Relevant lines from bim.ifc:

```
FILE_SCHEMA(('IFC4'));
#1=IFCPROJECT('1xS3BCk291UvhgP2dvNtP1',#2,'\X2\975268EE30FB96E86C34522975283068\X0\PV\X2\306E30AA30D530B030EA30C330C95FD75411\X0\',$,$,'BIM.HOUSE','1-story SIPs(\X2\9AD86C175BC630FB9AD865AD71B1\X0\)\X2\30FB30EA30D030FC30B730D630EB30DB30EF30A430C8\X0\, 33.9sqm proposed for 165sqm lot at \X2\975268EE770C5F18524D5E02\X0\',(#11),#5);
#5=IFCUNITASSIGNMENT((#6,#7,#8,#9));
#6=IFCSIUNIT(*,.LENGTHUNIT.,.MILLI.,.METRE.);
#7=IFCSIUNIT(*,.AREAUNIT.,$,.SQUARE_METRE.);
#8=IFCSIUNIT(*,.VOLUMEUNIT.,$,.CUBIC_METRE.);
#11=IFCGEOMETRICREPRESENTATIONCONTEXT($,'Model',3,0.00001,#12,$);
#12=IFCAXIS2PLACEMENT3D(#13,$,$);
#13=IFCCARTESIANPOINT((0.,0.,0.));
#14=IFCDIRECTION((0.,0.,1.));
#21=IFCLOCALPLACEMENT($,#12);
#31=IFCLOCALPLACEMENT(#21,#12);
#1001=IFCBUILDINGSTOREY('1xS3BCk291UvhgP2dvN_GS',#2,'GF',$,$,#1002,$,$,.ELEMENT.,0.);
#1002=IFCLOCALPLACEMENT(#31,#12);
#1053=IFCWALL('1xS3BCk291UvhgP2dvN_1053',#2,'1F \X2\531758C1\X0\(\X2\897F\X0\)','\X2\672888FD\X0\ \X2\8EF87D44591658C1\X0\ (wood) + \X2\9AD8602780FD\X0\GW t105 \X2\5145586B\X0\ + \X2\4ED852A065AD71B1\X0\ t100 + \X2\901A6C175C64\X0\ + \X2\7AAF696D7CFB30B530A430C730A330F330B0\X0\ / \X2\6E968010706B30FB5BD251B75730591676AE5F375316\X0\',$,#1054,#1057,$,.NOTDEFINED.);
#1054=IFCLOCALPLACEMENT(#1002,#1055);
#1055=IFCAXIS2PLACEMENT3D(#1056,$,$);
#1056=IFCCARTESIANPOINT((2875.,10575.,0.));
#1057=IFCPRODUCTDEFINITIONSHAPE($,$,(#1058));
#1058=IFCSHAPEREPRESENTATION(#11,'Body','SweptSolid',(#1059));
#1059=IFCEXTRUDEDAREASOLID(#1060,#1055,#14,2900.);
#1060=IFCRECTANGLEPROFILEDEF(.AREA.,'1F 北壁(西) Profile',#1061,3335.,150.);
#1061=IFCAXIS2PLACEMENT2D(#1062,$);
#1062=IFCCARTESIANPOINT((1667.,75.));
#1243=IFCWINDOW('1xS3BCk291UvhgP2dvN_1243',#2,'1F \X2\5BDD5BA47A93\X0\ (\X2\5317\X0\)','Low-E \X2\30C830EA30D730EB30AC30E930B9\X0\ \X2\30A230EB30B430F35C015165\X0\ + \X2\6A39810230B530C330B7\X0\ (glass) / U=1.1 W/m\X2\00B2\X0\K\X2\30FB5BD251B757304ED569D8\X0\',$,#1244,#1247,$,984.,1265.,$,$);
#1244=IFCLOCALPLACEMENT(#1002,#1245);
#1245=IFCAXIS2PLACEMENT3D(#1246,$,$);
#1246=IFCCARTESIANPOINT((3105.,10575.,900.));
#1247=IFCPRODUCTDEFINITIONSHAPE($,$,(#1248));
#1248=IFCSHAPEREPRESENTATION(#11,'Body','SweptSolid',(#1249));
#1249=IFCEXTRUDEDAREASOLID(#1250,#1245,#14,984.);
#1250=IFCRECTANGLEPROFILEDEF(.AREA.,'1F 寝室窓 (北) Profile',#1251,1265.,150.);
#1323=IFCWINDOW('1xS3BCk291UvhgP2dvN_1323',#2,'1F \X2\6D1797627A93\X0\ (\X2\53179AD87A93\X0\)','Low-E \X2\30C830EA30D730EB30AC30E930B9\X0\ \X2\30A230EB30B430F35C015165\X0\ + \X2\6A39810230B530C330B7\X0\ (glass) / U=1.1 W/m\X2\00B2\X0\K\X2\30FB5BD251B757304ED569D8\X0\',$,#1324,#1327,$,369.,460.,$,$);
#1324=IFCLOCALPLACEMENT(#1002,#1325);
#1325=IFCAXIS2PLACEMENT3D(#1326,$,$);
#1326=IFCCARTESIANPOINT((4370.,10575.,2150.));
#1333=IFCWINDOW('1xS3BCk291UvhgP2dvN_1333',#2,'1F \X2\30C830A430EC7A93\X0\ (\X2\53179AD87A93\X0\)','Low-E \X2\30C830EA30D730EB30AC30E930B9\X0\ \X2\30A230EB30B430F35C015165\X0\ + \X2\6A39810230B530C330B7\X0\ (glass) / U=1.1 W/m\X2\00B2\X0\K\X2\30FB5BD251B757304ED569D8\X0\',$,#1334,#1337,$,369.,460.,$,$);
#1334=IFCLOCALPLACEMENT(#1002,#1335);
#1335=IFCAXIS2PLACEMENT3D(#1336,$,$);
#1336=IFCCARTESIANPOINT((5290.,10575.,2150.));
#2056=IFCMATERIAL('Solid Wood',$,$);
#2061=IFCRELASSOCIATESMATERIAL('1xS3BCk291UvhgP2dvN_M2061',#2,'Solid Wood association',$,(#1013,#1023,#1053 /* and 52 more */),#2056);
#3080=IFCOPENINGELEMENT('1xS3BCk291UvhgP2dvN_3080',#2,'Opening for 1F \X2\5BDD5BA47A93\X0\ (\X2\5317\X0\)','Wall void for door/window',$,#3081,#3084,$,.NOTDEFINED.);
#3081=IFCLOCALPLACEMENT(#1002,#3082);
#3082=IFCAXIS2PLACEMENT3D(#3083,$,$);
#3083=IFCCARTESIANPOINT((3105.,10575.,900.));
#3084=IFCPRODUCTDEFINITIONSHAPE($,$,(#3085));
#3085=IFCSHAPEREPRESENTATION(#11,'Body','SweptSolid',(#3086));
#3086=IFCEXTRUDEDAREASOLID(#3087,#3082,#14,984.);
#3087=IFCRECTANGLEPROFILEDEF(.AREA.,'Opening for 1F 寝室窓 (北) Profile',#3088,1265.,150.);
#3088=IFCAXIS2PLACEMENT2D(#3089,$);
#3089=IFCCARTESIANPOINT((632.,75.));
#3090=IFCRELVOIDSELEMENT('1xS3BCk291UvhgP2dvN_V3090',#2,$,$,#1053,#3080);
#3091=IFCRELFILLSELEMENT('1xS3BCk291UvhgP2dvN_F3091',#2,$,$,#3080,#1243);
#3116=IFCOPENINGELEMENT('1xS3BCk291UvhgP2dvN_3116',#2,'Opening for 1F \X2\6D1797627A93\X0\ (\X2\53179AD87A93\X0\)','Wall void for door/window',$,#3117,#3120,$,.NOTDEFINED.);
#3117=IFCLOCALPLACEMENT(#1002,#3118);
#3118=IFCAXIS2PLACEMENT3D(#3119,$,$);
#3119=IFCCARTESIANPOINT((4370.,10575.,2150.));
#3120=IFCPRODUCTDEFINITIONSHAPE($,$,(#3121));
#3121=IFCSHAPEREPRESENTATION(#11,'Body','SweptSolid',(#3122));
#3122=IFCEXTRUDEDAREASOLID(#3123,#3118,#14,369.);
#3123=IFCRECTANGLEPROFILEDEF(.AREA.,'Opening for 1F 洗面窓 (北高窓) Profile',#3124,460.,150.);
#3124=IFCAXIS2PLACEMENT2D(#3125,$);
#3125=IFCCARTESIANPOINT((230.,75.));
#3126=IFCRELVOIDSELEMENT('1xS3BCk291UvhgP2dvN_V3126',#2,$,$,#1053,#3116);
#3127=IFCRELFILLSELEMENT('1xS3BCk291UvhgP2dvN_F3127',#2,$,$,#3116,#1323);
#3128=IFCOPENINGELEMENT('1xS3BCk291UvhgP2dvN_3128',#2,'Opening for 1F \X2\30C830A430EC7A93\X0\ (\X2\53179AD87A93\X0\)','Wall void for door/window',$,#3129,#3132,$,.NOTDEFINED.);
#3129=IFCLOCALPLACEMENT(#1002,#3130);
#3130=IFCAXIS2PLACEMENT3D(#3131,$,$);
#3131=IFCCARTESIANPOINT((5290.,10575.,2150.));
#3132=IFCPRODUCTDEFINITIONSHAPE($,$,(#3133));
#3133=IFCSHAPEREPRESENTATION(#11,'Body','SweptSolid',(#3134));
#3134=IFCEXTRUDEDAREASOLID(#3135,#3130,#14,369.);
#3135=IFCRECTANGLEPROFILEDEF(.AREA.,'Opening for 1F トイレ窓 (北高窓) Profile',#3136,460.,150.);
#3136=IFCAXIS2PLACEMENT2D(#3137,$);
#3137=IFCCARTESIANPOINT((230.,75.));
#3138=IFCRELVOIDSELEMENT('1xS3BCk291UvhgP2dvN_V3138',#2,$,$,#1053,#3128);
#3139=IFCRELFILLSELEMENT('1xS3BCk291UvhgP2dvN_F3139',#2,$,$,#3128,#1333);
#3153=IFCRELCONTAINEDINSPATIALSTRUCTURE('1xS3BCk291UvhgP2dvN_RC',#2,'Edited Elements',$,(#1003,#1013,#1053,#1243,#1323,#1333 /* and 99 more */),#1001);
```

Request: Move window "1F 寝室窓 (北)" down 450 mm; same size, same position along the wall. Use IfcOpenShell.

```python
import numpy as np
import ifcopenshell
import ifcopenshell.api.geometry
import ifcopenshell.util.placement
import ifcopenshell.util.unit

model = ifcopenshell.open("bim.ifc")
unit_scale = ifcopenshell.util.unit.calculate_unit_scale(model)

window = model.by_id(1243)
opening = window.FillsVoids[0].RelatingOpeningElement
dz = -450.0

shift = np.array([0.0, 0.0, dz])
# The window is not placed relative to its opening, so move both.
for product in (opening, window):
    matrix = ifcopenshell.util.placement.get_local_placement(product.ObjectPlacement)
    matrix[:3, 3] += shift
    ifcopenshell.api.geometry.edit_object_placement(model, product=product, matrix=matrix, is_si=False)

print(f"moved by {dz * unit_scale:+.3f} m")

model.write("bim_edited.ifc")
```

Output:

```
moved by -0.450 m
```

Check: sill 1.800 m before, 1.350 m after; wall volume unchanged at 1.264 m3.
